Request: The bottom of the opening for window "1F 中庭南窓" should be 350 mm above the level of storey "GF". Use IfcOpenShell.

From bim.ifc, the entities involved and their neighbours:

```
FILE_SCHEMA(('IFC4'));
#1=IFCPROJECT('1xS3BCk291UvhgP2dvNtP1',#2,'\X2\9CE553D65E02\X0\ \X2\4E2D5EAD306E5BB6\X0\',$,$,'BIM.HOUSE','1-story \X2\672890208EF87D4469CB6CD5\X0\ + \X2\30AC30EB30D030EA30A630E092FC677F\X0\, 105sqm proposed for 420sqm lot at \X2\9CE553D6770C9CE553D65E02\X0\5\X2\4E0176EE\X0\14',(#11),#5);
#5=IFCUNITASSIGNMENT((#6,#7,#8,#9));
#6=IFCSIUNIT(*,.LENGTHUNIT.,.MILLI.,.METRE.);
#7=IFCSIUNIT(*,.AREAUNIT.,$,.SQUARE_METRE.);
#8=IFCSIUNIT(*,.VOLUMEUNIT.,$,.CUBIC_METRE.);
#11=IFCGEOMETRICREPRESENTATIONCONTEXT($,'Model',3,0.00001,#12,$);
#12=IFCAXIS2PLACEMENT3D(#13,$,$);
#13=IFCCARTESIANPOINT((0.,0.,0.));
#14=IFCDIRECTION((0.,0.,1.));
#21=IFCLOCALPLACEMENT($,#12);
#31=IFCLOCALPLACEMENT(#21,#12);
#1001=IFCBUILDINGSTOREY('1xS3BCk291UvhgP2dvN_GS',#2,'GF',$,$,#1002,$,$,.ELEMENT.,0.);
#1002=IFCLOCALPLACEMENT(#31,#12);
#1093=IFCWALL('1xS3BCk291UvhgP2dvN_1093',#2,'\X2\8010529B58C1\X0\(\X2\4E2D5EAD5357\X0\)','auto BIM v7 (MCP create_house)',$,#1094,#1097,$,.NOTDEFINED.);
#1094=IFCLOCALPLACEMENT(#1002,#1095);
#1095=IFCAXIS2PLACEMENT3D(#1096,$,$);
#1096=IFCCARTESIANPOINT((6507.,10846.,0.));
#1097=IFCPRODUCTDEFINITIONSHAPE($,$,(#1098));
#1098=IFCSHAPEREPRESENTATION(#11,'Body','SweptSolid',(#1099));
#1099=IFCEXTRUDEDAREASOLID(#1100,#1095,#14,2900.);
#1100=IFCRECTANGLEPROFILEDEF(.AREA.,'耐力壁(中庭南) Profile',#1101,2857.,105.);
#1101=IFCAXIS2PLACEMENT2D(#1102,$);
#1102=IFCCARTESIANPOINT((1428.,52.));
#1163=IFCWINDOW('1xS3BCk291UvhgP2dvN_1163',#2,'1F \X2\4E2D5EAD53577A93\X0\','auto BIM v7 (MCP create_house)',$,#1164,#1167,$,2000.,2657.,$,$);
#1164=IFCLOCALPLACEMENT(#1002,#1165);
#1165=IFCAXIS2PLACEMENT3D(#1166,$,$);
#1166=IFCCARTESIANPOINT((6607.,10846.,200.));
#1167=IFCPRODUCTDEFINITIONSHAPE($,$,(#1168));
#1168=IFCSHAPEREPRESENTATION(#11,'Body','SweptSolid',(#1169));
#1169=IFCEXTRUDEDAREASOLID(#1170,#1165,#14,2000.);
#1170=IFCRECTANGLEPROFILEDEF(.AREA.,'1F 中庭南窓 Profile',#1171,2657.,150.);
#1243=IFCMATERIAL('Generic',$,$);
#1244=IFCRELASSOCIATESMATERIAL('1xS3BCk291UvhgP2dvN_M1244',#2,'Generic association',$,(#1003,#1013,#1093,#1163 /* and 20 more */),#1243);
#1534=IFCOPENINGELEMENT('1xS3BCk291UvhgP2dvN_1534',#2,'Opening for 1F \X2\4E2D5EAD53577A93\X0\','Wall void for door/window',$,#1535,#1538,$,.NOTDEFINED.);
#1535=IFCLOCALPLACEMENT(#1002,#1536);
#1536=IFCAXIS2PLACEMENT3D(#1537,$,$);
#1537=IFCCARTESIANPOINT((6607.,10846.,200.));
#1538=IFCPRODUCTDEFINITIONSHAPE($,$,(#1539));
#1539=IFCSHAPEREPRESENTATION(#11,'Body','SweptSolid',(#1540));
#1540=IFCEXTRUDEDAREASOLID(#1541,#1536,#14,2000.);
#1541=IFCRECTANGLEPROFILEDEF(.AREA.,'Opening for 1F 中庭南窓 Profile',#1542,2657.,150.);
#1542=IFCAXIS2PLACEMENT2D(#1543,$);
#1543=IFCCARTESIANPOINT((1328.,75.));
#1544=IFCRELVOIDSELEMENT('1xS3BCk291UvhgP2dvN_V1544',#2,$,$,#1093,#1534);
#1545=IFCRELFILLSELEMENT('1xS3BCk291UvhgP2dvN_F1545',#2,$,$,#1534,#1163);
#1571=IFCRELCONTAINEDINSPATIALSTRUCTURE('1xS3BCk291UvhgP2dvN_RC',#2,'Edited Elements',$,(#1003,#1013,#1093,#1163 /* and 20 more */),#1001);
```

```python
import numpy as np
import ifcopenshell
import ifcopenshell.api.geometry
import ifcopenshell.geom
import ifcopenshell.util.element
import ifcopenshell.util.placement
import ifcopenshell.util.shape
import ifcopenshell.util.unit

model = ifcopenshell.open("bim.ifc")
unit_scale = ifcopenshell.util.unit.calculate_unit_scale(model)

window = model.by_guid("1xS3BCk291UvhgP2dvN_1163")
opening = window.FillsVoids[0].RelatingOpeningElement
storey = ifcopenshell.util.element.get_container(window, ifc_class="IfcBuildingStorey")
level = ifcopenshell.util.placement.get_local_placement(storey.ObjectPlacement)[2, 3]

# The opening's origin need not be at the sill, so measure its lowest point.
shape = ifcopenshell.geom.create_shape(ifcopenshell.geom.settings(), opening)
bottom = ifcopenshell.util.shape.get_shape_bottom_elevation(shape, shape.geometry) / unit_scale
dz = level + 0.35 / unit_scale - bottom

shift = np.array([0.0, 0.0, dz])
# The window is not placed relative to its opening, so move both.
for product in (opening, window):
    matrix = ifcopenshell.util.placement.get_local_placement(product.ObjectPlacement)
    matrix[:3, 3] += shift
    ifcopenshell.api.geometry.edit_object_placement(model, product=product, matrix=matrix, is_si=False)

print(f"moved by {dz * unit_scale:+.3f} m")

model.write("bim_rev.ifc")
```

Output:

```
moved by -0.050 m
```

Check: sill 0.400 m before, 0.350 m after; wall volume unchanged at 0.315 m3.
